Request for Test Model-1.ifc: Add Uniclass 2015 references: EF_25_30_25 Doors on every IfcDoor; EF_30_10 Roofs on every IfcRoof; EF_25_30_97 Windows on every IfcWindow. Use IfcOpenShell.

First a look at what the model holds.

```python
import ifcopenshell

model = ifcopenshell.open("Test Model-1.ifc")
print(model.schema)
print("classifications:", [c.Name for c in model.by_type("IfcClassification")])
for ifc_class in ("IfcDoor", "IfcRoof", "IfcStair", "IfcWall", "IfcWindow"):
    print(ifc_class, len(model.by_type(ifc_class)))
```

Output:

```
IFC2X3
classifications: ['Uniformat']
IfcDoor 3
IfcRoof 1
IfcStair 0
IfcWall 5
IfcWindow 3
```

```python
import ifcopenshell
import ifcopenshell.api.classification

model = ifcopenshell.open("Test Model-1.ifc")

# IFC2X3 requires Source and Edition and has no link from the project to the system.
system = model.create_entity("IfcClassification", Source="NBS", Edition="2015", Name="Uniclass 2015")

codes = {
    "IfcDoor": ("EF_25_30_25", "Doors"),
    "IfcRoof": ("EF_30_10", "Roofs"),
    "IfcWindow": ("EF_25_30_97", "Windows"),
}
for ifc_class, (code, name) in codes.items():
    products = model.by_type(ifc_class)
    ifcopenshell.api.classification.add_reference(
        model, products=products, classification=system, identification=code, name=name
    )
    print(code, len(products))

model.write("Test Model-1_updated.ifc")
```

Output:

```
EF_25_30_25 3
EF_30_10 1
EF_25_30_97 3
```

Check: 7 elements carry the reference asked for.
